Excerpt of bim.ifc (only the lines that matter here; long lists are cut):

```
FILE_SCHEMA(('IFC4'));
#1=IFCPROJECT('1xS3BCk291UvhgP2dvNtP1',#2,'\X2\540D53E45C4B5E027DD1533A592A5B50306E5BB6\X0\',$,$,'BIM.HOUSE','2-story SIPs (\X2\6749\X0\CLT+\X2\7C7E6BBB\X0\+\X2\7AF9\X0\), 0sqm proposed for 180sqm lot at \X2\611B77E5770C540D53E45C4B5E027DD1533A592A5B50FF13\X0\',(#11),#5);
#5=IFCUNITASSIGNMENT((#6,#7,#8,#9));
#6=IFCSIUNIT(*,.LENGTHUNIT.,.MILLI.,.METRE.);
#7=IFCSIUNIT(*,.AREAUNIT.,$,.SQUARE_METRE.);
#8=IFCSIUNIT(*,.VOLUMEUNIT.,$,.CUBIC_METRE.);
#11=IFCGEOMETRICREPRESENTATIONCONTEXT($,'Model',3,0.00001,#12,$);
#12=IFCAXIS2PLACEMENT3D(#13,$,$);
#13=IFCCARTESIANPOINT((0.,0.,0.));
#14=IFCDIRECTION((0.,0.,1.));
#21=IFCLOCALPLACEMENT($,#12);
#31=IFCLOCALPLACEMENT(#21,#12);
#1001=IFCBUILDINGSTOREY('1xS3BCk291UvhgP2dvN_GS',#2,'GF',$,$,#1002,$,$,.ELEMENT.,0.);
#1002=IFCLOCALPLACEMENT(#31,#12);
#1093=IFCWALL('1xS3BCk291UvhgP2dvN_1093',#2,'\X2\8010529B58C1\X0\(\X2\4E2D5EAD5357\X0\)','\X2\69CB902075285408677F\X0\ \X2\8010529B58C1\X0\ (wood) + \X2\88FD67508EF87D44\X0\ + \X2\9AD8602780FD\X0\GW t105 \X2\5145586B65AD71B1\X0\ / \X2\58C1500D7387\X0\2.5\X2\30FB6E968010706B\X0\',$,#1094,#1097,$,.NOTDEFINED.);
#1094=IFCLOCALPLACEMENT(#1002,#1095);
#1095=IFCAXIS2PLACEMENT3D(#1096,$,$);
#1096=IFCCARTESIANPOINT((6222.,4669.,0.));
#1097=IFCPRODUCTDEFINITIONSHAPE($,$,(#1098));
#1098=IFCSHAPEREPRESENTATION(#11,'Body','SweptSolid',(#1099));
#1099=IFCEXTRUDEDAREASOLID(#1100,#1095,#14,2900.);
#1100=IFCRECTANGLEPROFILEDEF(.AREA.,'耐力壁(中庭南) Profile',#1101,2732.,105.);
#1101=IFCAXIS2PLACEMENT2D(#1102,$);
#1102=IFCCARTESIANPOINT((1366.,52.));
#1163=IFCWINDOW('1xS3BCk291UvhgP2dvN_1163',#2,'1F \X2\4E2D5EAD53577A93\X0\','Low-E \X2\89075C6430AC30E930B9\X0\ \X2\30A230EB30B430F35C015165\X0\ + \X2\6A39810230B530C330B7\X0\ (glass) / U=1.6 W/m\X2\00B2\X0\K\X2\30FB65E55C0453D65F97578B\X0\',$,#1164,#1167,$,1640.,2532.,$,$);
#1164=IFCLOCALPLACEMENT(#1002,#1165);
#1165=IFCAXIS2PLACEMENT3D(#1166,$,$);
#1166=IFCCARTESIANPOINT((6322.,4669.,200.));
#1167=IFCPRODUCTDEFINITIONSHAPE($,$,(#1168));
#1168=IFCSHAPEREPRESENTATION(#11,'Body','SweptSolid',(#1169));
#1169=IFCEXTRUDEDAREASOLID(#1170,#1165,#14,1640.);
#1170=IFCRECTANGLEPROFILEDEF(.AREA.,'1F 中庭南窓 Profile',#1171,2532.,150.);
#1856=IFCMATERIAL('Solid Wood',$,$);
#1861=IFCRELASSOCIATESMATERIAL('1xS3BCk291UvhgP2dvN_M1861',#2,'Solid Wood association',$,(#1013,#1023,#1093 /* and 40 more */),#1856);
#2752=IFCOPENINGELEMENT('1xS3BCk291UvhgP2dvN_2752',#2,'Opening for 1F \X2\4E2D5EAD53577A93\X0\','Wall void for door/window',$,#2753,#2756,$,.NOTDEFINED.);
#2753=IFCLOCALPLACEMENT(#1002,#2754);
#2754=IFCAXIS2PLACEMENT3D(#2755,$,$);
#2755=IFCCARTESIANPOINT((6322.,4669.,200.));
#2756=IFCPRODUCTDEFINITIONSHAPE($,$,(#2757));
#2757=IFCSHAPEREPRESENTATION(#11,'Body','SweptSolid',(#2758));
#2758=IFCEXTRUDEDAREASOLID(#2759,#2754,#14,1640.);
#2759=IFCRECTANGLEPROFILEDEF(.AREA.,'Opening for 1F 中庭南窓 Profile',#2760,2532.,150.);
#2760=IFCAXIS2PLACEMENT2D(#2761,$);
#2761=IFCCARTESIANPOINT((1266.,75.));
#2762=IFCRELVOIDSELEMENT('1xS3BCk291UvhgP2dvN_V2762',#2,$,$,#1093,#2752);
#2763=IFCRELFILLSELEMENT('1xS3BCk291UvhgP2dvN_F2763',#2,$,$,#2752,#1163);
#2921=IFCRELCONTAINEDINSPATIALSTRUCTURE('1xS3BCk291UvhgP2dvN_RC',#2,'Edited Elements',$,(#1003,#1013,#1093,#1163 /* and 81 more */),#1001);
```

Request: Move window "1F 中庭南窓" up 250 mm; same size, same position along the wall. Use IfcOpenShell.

```python
import numpy as np
import ifcopenshell
import ifcopenshell.api.geometry
import ifcopenshell.util.placement
import ifcopenshell.util.unit

model = ifcopenshell.open("bim.ifc")
unit_scale = ifcopenshell.util.unit.calculate_unit_scale(model)

window = model.by_id(1163)
opening = window.FillsVoids[0].RelatingOpeningElement
dz = 0.25 / unit_scale

shift = np.array([0.0, 0.0, dz])
# The window is not placed relative to its opening, so move both.
for product in (opening, window):
    matrix = ifcopenshell.util.placement.get_local_placement(product.ObjectPlacement)
    matrix[:3, 3] += shift
    ifcopenshell.api.geometry.edit_object_placement(model, product=product, matrix=matrix, is_si=False)

print(f"moved by {dz * unit_scale:+.3f} m")

model.write("bim_updated.ifc")
```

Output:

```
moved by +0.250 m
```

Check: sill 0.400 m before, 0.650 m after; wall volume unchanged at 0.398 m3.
